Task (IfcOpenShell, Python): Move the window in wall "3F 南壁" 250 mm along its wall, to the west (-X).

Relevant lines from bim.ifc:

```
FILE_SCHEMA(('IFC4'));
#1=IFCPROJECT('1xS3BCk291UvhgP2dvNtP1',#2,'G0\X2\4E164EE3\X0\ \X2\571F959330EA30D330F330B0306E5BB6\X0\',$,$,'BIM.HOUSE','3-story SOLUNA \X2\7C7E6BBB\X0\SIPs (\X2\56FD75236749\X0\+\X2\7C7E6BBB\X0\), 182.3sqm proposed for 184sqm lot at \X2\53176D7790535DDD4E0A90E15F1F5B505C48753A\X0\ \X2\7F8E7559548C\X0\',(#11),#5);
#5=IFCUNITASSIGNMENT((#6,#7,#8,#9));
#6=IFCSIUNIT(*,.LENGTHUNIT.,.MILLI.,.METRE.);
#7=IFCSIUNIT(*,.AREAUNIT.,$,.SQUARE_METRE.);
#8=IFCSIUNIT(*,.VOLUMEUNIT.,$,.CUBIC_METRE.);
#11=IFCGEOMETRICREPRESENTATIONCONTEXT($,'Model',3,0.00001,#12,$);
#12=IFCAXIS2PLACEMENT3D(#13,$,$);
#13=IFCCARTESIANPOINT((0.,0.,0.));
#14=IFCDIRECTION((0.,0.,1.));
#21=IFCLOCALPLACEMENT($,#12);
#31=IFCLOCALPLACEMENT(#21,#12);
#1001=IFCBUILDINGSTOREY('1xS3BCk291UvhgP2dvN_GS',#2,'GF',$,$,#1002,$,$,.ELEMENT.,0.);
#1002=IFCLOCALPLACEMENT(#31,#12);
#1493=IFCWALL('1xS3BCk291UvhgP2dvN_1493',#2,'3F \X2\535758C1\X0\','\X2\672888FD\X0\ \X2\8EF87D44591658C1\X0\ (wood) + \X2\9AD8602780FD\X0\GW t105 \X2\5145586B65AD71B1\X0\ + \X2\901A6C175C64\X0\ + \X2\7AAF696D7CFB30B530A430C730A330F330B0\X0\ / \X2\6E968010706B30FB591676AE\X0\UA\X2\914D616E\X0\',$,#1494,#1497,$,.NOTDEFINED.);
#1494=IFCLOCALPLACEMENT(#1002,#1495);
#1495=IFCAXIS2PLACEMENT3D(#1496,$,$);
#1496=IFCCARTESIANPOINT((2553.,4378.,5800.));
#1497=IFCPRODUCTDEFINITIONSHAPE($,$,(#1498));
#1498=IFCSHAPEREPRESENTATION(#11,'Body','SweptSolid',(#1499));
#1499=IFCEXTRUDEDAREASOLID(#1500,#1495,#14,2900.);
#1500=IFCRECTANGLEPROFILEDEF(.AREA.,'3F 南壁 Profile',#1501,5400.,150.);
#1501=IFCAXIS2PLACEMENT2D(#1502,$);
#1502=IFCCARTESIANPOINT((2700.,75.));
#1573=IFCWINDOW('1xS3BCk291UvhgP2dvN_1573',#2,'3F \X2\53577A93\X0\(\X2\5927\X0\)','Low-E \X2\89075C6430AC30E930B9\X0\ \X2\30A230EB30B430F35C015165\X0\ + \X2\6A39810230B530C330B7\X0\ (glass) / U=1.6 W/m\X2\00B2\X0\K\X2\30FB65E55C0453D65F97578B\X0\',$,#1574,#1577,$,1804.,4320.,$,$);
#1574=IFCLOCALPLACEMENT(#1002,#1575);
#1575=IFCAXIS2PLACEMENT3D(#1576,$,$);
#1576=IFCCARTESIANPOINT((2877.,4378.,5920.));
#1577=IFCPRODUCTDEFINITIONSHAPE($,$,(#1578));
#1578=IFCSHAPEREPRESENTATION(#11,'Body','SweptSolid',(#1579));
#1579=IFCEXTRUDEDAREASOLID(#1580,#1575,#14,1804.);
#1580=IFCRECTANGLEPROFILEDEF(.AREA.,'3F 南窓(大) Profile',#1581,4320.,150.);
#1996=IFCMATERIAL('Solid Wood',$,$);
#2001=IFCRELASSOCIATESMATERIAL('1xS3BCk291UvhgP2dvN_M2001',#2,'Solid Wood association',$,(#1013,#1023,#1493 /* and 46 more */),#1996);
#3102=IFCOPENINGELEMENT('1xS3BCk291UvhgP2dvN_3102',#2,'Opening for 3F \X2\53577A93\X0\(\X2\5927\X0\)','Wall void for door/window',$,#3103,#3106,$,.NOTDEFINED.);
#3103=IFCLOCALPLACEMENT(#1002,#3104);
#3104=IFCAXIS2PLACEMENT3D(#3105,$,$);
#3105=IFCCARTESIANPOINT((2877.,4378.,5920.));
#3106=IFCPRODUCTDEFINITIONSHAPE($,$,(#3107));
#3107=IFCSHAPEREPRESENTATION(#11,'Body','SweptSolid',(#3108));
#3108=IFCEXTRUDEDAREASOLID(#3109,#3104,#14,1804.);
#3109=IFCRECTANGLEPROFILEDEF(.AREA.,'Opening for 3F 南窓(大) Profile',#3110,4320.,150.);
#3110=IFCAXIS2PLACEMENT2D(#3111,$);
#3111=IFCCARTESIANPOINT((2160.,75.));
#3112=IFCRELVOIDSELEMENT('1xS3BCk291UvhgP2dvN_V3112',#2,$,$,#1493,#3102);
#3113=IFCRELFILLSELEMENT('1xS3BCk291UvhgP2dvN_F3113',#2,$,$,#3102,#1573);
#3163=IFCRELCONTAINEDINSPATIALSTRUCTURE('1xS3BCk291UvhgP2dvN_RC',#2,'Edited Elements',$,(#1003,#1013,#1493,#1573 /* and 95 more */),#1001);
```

```python
import ifcopenshell
import ifcopenshell.api.geometry
import ifcopenshell.util.placement
import ifcopenshell.util.unit

model = ifcopenshell.open("bim.ifc")
unit_scale = ifcopenshell.util.unit.calculate_unit_scale(model)

window = model.by_guid("1xS3BCk291UvhgP2dvN_1573")
opening = window.FillsVoids[0].RelatingOpeningElement
wall = opening.VoidsElements[0].RelatingBuildingElement

wall_matrix = ifcopenshell.util.placement.get_local_placement(wall.ObjectPlacement)
shift = wall_matrix[:3, 0] * -0.25 / unit_scale
before = ifcopenshell.util.placement.get_local_placement(window.ObjectPlacement)[:3, 3].copy()

# The window is not placed relative to its opening, so move both.
for product in (opening, window):
    matrix = ifcopenshell.util.placement.get_local_placement(product.ObjectPlacement)
    matrix[:3, 3] += shift
    ifcopenshell.api.geometry.edit_object_placement(model, product=product, matrix=matrix, is_si=False)

after = ifcopenshell.util.placement.get_local_placement(window.ObjectPlacement)[:3, 3]
print("window moved by", (after - before).round(3) + 0.0)

model.write("bim_edited.ifc")
```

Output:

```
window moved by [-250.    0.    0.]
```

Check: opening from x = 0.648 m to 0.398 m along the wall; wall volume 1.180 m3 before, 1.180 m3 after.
